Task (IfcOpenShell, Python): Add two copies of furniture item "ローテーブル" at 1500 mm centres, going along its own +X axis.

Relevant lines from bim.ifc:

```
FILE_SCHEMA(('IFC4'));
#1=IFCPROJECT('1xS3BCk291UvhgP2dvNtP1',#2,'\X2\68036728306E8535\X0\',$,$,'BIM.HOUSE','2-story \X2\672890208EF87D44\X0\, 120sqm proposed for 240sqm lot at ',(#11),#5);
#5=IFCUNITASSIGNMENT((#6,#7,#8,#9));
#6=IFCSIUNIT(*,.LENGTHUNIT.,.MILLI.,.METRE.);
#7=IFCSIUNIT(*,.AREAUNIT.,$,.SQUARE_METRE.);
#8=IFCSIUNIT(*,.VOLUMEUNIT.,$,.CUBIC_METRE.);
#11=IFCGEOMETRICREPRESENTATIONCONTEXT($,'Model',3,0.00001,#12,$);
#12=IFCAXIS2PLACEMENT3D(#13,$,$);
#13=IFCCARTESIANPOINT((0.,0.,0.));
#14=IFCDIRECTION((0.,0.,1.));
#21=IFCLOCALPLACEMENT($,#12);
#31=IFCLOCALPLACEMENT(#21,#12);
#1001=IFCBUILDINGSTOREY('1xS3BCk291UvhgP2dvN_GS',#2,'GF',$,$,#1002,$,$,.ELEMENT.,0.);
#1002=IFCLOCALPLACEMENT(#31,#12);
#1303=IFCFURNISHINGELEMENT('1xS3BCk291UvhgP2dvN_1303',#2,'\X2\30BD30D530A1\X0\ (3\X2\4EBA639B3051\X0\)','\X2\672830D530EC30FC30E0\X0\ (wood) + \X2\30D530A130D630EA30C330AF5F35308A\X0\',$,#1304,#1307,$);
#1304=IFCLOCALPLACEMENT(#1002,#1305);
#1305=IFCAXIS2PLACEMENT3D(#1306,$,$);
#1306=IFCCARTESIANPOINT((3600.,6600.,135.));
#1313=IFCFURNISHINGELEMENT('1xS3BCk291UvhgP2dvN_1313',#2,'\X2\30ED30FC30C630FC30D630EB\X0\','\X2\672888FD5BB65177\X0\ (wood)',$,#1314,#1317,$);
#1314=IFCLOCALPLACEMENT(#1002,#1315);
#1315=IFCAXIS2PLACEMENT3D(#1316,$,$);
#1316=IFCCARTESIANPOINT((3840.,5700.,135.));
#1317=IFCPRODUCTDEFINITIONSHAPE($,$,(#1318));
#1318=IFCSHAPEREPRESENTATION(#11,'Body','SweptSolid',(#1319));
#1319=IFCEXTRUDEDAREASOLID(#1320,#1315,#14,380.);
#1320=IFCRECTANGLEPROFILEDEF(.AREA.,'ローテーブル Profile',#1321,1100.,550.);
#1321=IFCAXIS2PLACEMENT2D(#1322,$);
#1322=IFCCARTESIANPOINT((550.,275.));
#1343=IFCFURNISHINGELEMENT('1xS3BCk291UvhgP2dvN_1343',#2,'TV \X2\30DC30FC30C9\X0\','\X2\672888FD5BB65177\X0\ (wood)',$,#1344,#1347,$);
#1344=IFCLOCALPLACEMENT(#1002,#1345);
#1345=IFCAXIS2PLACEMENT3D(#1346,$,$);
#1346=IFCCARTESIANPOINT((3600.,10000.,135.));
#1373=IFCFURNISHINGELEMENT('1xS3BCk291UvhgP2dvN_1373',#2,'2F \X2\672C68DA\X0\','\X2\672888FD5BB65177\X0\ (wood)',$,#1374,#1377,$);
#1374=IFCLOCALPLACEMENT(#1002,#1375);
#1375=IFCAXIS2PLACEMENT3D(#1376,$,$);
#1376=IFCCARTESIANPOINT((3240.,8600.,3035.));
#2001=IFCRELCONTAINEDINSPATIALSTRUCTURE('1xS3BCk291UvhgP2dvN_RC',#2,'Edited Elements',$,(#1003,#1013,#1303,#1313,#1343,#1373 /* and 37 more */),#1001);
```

```python
import ifcopenshell
import ifcopenshell.api.geometry
import ifcopenshell.api.root
import ifcopenshell.util.element
import ifcopenshell.util.placement

model = ifcopenshell.open("bim.ifc")


def reuse_history(source, copy):
    """copy_class also copies each property set's owner history, people and application; keep the originals."""
    for rel in copy.IsDefinedBy:
        if rel.is_a("IfcRelDefinesByProperties") and (history := rel.RelatingPropertyDefinition.OwnerHistory):
            rel.RelatingPropertyDefinition.OwnerHistory = source.OwnerHistory
            ifcopenshell.util.element.remove_deep2(model, history)


source = model.by_guid("1xS3BCk291UvhgP2dvN_1313")
base = ifcopenshell.util.placement.get_local_placement(source.ObjectPlacement)
step = base[:3, 0] * 1500.0

for i in range(1, 3):
    copy = ifcopenshell.api.root.copy_class(model, product=source)
    copy.Representation = ifcopenshell.util.element.copy_deep(
        model, source.Representation, exclude=["IfcGeometricRepresentationContext", "IfcRepresentationMap"]
    )
    reuse_history(source, copy)
    matrix = base.copy()
    matrix[:3, 3] += i * step
    print("added at", matrix[:3, 3].round(3) + 0.0)
    ifcopenshell.api.geometry.edit_object_placement(model, product=copy, matrix=matrix, is_si=False)

model.write("bim_rev.ifc")
```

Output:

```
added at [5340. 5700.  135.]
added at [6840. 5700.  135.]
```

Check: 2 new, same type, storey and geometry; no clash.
